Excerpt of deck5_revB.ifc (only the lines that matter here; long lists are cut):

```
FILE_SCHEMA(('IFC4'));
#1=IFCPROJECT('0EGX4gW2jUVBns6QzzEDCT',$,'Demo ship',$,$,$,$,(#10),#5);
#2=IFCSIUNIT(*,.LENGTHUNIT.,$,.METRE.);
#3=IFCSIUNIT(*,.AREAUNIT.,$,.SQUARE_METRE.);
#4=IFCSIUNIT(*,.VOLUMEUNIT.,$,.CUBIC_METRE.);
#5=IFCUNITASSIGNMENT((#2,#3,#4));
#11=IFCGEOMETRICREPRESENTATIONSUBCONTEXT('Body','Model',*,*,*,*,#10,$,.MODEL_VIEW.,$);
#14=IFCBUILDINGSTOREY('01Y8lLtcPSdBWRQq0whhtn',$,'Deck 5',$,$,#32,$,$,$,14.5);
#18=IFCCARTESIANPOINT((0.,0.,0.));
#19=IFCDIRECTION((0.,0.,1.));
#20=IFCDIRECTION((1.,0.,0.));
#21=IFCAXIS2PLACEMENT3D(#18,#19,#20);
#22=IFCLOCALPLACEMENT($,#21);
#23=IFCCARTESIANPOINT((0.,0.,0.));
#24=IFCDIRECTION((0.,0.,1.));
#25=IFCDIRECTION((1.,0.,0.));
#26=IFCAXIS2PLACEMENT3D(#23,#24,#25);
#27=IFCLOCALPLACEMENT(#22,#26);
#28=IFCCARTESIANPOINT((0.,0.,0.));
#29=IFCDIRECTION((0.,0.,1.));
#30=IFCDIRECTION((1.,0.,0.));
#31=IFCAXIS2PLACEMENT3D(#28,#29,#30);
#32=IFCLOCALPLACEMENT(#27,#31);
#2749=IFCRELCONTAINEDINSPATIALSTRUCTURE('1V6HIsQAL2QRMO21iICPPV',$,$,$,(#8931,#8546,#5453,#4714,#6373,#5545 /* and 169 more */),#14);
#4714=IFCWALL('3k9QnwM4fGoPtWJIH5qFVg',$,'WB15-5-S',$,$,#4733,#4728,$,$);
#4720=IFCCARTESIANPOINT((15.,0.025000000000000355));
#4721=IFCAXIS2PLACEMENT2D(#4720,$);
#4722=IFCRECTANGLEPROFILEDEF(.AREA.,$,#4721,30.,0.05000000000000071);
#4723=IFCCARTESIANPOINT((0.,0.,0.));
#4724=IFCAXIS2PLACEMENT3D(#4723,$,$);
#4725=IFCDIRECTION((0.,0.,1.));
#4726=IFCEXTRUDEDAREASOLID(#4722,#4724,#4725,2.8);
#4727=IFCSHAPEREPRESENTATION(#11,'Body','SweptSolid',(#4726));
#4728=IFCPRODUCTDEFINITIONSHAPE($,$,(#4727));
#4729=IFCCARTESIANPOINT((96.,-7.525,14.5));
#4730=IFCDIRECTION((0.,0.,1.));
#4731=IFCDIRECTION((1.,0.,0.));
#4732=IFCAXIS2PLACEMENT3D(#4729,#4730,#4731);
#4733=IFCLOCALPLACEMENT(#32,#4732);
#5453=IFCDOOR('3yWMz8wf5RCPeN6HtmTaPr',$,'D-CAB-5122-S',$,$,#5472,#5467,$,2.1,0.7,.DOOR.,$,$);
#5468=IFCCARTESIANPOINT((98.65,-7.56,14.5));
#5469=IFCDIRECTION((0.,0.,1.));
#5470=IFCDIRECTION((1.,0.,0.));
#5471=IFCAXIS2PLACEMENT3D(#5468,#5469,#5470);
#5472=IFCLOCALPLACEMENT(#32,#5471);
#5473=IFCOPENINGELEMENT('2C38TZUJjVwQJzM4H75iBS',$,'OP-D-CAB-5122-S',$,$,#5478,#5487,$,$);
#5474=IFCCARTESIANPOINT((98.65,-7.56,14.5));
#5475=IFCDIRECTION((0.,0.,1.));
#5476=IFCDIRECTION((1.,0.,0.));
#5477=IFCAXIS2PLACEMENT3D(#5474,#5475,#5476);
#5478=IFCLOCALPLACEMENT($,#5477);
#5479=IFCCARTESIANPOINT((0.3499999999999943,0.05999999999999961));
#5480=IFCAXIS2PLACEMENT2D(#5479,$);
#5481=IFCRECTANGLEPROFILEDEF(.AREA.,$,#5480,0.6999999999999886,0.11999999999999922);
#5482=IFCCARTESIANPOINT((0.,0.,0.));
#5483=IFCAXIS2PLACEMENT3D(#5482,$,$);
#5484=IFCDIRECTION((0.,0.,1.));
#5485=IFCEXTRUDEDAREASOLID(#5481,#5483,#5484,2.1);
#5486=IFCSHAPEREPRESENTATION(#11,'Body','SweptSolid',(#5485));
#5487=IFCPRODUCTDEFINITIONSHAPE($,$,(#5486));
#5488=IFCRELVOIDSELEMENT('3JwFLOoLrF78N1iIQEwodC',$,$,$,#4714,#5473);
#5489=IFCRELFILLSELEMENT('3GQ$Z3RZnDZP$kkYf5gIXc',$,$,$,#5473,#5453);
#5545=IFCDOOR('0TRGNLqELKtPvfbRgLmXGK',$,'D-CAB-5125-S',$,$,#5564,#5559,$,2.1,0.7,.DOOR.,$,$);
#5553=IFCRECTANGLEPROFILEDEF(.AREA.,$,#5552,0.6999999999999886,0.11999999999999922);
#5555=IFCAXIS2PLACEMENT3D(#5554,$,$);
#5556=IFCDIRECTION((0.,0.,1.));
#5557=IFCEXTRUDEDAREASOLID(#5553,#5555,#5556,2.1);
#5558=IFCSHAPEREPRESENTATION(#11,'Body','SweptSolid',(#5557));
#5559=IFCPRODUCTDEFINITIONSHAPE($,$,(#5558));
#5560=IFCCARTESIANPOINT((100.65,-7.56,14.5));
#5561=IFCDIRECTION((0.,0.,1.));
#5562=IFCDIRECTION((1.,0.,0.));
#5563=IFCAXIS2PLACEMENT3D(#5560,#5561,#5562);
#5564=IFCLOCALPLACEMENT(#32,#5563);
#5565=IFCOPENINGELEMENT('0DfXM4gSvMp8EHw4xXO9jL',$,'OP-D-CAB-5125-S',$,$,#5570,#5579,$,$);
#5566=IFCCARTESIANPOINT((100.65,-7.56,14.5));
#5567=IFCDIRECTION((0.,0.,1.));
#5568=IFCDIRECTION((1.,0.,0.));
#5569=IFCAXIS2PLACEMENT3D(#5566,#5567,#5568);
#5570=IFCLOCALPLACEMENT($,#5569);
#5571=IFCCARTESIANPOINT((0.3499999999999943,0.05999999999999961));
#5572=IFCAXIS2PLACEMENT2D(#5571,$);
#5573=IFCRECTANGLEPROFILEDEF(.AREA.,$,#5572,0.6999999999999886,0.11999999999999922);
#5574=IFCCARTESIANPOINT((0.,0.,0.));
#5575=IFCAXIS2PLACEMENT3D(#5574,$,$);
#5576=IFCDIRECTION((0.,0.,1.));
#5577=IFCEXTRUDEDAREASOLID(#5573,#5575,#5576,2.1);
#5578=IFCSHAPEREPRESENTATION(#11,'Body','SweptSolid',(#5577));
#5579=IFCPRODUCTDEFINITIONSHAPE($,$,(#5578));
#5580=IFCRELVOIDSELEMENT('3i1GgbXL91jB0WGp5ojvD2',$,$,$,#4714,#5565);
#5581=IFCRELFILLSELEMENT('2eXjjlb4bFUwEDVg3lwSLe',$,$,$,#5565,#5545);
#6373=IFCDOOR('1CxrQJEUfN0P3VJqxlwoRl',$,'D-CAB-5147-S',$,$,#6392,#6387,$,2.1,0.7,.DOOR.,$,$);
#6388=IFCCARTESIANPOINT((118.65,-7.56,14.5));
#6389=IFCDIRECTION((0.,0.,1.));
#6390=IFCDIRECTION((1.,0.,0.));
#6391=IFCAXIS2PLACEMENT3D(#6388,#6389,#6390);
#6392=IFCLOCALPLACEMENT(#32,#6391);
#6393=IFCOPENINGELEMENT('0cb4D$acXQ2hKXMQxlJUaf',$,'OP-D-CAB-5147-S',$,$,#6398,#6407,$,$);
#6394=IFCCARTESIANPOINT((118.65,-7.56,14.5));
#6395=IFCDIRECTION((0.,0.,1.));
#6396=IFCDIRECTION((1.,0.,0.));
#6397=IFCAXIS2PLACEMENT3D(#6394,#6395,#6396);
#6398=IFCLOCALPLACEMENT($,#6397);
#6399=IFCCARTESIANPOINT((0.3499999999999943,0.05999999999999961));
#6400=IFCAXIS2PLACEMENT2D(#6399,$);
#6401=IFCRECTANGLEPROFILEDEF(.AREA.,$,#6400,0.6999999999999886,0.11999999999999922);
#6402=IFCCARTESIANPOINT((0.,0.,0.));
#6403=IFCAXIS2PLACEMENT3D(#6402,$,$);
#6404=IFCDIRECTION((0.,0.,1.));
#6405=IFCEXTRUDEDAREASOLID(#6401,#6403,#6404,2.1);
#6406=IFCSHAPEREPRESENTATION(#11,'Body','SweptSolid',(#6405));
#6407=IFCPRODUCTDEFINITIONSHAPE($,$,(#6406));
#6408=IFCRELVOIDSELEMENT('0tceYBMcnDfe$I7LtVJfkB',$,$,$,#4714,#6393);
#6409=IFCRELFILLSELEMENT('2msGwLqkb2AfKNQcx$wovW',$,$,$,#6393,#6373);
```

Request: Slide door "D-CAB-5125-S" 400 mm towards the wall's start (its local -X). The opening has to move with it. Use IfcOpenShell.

```python
import ifcopenshell
import ifcopenshell.api.geometry
import ifcopenshell.util.placement
import ifcopenshell.util.unit

model = ifcopenshell.open("deck5_revB.ifc")
unit_scale = ifcopenshell.util.unit.calculate_unit_scale(model)

door = model.by_guid("0TRGNLqELKtPvfbRgLmXGK")
opening = door.FillsVoids[0].RelatingOpeningElement
wall = opening.VoidsElements[0].RelatingBuildingElement

wall_matrix = ifcopenshell.util.placement.get_local_placement(wall.ObjectPlacement)
shift = wall_matrix[:3, 0] * -0.4 / unit_scale
before = ifcopenshell.util.placement.get_local_placement(door.ObjectPlacement)[:3, 3].copy()

# The door is not placed relative to its opening, so move both.
for product in (opening, door):
    matrix = ifcopenshell.util.placement.get_local_placement(product.ObjectPlacement)
    matrix[:3, 3] += shift
    ifcopenshell.api.geometry.edit_object_placement(model, product=product, matrix=matrix, is_si=False)

after = ifcopenshell.util.placement.get_local_placement(door.ObjectPlacement)[:3, 3]
print("door moved by", (after - before).round(3) + 0.0)

model.write("deck5_revB_v2.ifc")
```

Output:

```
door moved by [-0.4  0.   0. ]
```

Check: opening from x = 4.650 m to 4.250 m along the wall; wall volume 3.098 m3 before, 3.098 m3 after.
